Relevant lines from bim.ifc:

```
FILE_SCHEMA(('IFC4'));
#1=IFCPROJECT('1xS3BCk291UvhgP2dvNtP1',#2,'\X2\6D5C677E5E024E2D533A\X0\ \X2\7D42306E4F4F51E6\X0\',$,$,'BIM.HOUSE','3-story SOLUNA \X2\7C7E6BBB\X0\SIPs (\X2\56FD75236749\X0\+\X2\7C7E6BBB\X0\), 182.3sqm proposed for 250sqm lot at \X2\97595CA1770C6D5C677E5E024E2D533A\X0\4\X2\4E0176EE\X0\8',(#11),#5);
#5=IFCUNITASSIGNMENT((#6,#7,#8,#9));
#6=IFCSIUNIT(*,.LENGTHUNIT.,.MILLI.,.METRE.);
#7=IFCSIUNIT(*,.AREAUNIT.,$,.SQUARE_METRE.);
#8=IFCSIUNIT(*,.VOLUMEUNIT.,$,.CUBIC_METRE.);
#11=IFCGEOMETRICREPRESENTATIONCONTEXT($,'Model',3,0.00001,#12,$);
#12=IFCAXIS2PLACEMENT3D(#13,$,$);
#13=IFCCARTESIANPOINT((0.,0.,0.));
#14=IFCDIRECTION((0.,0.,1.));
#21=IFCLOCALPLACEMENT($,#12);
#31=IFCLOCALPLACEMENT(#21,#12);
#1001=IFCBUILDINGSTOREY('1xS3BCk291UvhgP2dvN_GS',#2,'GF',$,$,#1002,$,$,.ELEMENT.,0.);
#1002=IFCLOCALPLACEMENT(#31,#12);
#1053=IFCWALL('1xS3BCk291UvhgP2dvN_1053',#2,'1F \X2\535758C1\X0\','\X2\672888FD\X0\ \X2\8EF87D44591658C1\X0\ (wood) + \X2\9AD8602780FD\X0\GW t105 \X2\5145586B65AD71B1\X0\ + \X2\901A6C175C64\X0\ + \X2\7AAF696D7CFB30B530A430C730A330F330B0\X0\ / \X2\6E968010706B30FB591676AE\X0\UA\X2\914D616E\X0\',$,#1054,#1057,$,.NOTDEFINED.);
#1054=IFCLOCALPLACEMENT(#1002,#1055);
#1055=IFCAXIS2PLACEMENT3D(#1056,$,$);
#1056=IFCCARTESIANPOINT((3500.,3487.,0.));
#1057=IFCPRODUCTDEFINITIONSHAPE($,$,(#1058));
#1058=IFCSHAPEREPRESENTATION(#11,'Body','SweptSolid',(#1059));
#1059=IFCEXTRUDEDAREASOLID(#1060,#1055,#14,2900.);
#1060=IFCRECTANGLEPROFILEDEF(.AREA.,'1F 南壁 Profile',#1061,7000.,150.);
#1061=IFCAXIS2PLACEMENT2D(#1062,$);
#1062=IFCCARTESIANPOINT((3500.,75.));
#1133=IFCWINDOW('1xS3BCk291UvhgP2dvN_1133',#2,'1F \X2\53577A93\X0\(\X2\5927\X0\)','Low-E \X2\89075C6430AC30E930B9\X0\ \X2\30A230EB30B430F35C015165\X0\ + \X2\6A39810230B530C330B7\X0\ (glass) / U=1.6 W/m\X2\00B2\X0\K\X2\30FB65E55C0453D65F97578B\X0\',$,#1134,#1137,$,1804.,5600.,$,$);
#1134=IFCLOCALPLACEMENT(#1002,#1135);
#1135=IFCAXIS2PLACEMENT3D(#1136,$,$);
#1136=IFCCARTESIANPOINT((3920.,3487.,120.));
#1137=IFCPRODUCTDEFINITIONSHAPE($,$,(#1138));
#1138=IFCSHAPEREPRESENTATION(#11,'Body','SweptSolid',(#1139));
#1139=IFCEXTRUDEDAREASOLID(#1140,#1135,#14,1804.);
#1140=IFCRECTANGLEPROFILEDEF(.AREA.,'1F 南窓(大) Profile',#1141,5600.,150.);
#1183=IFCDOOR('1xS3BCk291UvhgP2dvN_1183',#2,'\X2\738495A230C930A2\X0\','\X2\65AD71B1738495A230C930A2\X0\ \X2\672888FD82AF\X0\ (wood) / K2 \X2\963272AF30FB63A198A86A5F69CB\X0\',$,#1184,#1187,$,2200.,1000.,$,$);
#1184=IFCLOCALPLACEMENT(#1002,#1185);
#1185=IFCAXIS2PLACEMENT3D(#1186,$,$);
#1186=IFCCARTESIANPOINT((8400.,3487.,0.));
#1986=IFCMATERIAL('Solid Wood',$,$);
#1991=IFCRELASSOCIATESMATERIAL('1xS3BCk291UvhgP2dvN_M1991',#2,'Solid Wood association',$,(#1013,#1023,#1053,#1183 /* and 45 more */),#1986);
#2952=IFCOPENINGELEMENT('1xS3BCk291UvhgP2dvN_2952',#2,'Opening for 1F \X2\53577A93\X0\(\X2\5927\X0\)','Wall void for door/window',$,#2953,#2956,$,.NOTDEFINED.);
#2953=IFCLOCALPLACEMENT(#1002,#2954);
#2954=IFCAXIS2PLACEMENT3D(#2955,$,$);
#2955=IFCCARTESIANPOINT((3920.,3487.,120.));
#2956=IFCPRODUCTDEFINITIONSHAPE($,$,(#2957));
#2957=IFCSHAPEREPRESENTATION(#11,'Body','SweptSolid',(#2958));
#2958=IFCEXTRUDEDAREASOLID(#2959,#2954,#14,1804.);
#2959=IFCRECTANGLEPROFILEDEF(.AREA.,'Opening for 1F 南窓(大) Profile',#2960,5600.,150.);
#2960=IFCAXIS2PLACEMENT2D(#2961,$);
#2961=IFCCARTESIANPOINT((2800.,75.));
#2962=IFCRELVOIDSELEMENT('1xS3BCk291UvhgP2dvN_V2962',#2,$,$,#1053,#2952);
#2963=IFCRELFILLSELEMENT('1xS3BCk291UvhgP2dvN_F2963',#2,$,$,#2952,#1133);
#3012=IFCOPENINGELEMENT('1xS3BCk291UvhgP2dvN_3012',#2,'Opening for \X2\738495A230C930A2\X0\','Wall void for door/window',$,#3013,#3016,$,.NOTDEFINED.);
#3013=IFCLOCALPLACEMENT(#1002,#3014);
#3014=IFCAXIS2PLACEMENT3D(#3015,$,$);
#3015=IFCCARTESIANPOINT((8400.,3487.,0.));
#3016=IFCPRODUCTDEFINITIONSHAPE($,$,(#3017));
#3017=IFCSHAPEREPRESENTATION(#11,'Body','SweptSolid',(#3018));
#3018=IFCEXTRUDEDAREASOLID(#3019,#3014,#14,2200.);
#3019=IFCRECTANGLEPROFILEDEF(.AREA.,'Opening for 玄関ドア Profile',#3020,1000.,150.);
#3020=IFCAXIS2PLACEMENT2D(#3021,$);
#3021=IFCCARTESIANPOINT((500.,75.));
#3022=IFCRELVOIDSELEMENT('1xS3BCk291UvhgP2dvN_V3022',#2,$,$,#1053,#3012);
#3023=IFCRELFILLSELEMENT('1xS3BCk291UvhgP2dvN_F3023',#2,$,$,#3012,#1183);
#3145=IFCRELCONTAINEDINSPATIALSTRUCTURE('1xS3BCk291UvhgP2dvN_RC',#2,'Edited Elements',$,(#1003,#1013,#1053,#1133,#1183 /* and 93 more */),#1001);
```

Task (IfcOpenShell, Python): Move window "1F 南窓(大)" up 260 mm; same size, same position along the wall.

```python
import numpy as np
import ifcopenshell
import ifcopenshell.api.geometry
import ifcopenshell.util.placement
import ifcopenshell.util.unit

model = ifcopenshell.open("bim.ifc")
unit_scale = ifcopenshell.util.unit.calculate_unit_scale(model)

window = model.by_guid("1xS3BCk291UvhgP2dvN_1133")
opening = window.FillsVoids[0].RelatingOpeningElement
dz = 260.0

shift = np.array([0.0, 0.0, dz])
# The window is not placed relative to its opening, so move both.
for product in (opening, window):
    matrix = ifcopenshell.util.placement.get_local_placement(product.ObjectPlacement)
    matrix[:3, 3] += shift
    ifcopenshell.api.geometry.edit_object_placement(model, product=product, matrix=matrix, is_si=False)

print(f"moved by {dz * unit_scale:+.3f} m")

model.write("bim_v2.ifc")
```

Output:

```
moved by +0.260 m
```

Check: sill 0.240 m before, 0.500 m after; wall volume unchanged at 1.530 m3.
